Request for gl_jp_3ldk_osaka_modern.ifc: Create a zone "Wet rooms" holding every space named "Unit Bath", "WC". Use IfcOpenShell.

First a look at what the model holds.

```python
import ifcopenshell

model = ifcopenshell.open("gl_jp_3ldk_osaka_modern.ifc")
print(model.schema)
seen = {}
for space in model.by_type("IfcSpace"):
    seen[space.LongName] = seen.get(space.LongName, 0) + 1
for name, count in sorted(seen.items(), key=str):
    print(count, "x", name)
print("zones:", [z.Name for z in model.by_type("IfcZone")][:20])
```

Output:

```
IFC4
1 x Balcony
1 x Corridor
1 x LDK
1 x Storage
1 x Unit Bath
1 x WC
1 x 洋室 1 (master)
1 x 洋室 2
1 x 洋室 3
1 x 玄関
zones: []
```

```python
import ifcopenshell
import ifcopenshell.api.group
import ifcopenshell.api.root

model = ifcopenshell.open("gl_jp_3ldk_osaka_modern.ifc")

names = {"Unit Bath", "WC"}
spaces = [s for s in model.by_type("IfcSpace") if s.LongName in names]

zone = ifcopenshell.api.root.create_entity(model, ifc_class="IfcZone", name="Wet rooms")
ifcopenshell.api.group.assign_group(model, products=spaces, group=zone)
print(len(spaces), "spaces in", zone.Name)

model.write("gl_jp_3ldk_osaka_modern_rev.ifc")
```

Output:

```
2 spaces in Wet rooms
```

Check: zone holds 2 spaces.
